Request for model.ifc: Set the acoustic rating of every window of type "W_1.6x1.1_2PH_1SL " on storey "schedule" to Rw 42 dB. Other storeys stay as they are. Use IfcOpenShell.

First a look at what the model holds.

```python
import ifcopenshell
import ifcopenshell.util.element

model = ifcopenshell.open("model.ifc")
print(model.schema)
storey = next(s for s in model.by_type("IfcBuildingStorey") if s.Name == "schedule")
windows = [e for e in ifcopenshell.util.element.get_decomposition(storey) if e.is_a("IfcWindow")]
seen = {}
for e in windows:
    element_type = ifcopenshell.util.element.get_type(e)
    key = (element_type.Name if element_type != e and element_type else None, ifcopenshell.util.element.get_pset(e, "Pset_WindowCommon", "AcousticRating"))
    seen[key] = seen.get(key, 0) + 1
for (name, value), count in sorted(seen.items(), key=str):
    print(count, "x", name, "|", value)
```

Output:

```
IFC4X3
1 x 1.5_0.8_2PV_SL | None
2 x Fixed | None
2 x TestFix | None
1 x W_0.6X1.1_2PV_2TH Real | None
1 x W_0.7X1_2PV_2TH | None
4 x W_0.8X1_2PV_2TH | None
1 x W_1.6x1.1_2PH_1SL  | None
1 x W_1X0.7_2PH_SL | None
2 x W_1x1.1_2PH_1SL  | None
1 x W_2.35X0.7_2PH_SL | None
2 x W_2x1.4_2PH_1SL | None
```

```python
import ifcopenshell
import ifcopenshell.api.pset
import ifcopenshell.util.element

model = ifcopenshell.open("model.ifc")

storey = next(s for s in model.by_type("IfcBuildingStorey") if s.Name == "schedule")
windows = [e for e in ifcopenshell.util.element.get_decomposition(storey) if e.is_a("IfcWindow")]

count = 0
for e in windows:
    element_type = ifcopenshell.util.element.get_type(e)
    if element_type in (None, e) or element_type.Name != "W_1.6x1.1_2PH_1SL ":
        continue
    # add_pset returns the element's existing set when there is one.
    pset = ifcopenshell.api.pset.add_pset(model, product=e, name="Pset_WindowCommon")
    ifcopenshell.api.pset.edit_pset(model, pset=pset, properties={"AcousticRating": "Rw 42 dB"})
    count += 1

print(count, "windows updated")

model.write("model_v2.ifc")
```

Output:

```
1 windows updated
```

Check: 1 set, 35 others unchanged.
